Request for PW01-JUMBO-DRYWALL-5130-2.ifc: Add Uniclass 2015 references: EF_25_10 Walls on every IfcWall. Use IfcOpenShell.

First a look at what the model holds.

```python
import ifcopenshell

model = ifcopenshell.open("PW01-JUMBO-DRYWALL-5130-2.ifc")
print(model.schema)
print("classifications:", [c.Name for c in model.by_type("IfcClassification")])
for ifc_class in ("IfcDoor", "IfcRoof", "IfcStair", "IfcWall", "IfcWindow"):
    print(ifc_class, len(model.by_type(ifc_class)))
```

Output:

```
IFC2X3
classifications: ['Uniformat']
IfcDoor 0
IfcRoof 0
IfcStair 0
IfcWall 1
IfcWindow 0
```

```python
import ifcopenshell
import ifcopenshell.api.classification

model = ifcopenshell.open("PW01-JUMBO-DRYWALL-5130-2.ifc")

# IFC2X3 requires Source and Edition and has no link from the project to the system.
system = model.create_entity("IfcClassification", Source="NBS", Edition="2015", Name="Uniclass 2015")

codes = {
    "IfcWall": ("EF_25_10", "Walls"),
}
for ifc_class, (code, name) in codes.items():
    products = model.by_type(ifc_class)
    ifcopenshell.api.classification.add_reference(
        model, products=products, classification=system, identification=code, name=name
    )
    print(code, len(products))

model.write("PW01-JUMBO-DRYWALL-5130-2_v2.ifc")
```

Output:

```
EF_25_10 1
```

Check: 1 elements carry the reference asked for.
